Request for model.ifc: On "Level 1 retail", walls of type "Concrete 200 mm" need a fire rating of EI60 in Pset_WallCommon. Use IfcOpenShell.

First a look at what the model holds.

```python
import ifcopenshell
import ifcopenshell.util.element

model = ifcopenshell.open("model.ifc")
print(model.schema)
storey = next(s for s in model.by_type("IfcBuildingStorey") if s.Name == "Level 1 retail")
walls = [e for e in ifcopenshell.util.element.get_decomposition(storey) if e.is_a("IfcWall")]
seen = {}
for e in walls:
    element_type = ifcopenshell.util.element.get_type(e)
    key = (element_type.Name if element_type != e and element_type else None, ifcopenshell.util.element.get_pset(e, "Pset_WallCommon", "FireRating"))
    seen[key] = seen.get(key, 0) + 1
for (name, value), count in sorted(seen.items(), key=str):
    print(count, "x", name, "|", value)
```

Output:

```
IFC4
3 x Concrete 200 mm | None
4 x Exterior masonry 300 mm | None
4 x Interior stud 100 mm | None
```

```python
import ifcopenshell
import ifcopenshell.api.pset
import ifcopenshell.util.element

model = ifcopenshell.open("model.ifc")

storey = next(s for s in model.by_type("IfcBuildingStorey") if s.Name == "Level 1 retail")
walls = [e for e in ifcopenshell.util.element.get_decomposition(storey) if e.is_a("IfcWall")]

count = 0
for e in walls:
    element_type = ifcopenshell.util.element.get_type(e)
    if element_type in (None, e) or element_type.Name != "Concrete 200 mm":
        continue
    # add_pset returns the element's existing set when there is one.
    pset = ifcopenshell.api.pset.add_pset(model, product=e, name="Pset_WallCommon")
    ifcopenshell.api.pset.edit_pset(model, pset=pset, properties={"FireRating": "EI60"})
    count += 1

print(count, "walls updated")

model.write("model_rev.ifc")
```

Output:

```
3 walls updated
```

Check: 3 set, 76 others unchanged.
